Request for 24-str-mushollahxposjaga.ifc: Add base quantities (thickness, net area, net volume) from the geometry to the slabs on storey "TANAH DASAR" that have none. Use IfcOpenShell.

First a look at what the model holds.

```python
import ifcopenshell
import ifcopenshell.util.element
import ifcopenshell.util.unit

model = ifcopenshell.open("24-str-mushollahxposjaga.ifc")
print(model.schema)
for unit_type in ("LENGTHUNIT", "AREAUNIT", "VOLUMEUNIT"):
    print(unit_type, ifcopenshell.util.unit.calculate_unit_scale(model, unit_type))
storey = next(s for s in model.by_type("IfcBuildingStorey") if s.Name == "TANAH DASAR")
slabs = [e for e in ifcopenshell.util.element.get_decomposition(storey) if e.is_a("IfcSlab")]
for e in sorted(slabs, key=lambda e: e.id()):
    print(e.id(), e.is_a(), e.Name, list(ifcopenshell.util.element.get_psets(e, qtos_only=True)), sep=" | ")
```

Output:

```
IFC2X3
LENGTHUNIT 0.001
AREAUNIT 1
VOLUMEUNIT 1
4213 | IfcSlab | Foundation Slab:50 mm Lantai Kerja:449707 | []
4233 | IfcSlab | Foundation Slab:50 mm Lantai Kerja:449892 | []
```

```python
import ifcopenshell
import ifcopenshell.api.pset
import ifcopenshell.geom
import ifcopenshell.util.element
import ifcopenshell.util.shape
import ifcopenshell.util.unit

model = ifcopenshell.open("24-str-mushollahxposjaga.ifc")
unit_scale = ifcopenshell.util.unit.calculate_unit_scale(model)
area_scale = ifcopenshell.util.unit.calculate_unit_scale(model, "AREAUNIT")
volume_scale = ifcopenshell.util.unit.calculate_unit_scale(model, "VOLUMEUNIT")
settings = ifcopenshell.geom.settings()

storey = next(s for s in model.by_type("IfcBuildingStorey") if s.Name == "TANAH DASAR")
slabs = [e for e in ifcopenshell.util.element.get_decomposition(storey) if e.is_a("IfcSlab")]

for e in sorted(slabs, key=lambda e: e.id()):
    if ifcopenshell.util.element.get_psets(e, qtos_only=True, should_inherit=False):
        continue
    # Geometry comes back in metres, in the element's own axes.
    shape = ifcopenshell.geom.create_shape(settings, e)
    values = {
        "Width": ifcopenshell.util.shape.get_z(shape.geometry) / unit_scale,
        "NetArea": ifcopenshell.util.shape.get_footprint_area(shape.geometry) / area_scale,
        "NetVolume": ifcopenshell.util.shape.get_volume(shape.geometry) / volume_scale,
    }
    qto = ifcopenshell.api.pset.add_qto(model, product=e, name="BaseQuantities")
    ifcopenshell.api.pset.edit_qto(model, qto=qto, properties=values)
    print(e.id(), {k: round(v, 3) for k, v in values.items()})

model.write("24-str-mushollahxposjaga_rev.ifc")
```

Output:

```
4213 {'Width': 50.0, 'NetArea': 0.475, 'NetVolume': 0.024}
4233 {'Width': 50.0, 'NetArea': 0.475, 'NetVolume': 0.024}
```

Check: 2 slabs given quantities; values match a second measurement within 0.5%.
